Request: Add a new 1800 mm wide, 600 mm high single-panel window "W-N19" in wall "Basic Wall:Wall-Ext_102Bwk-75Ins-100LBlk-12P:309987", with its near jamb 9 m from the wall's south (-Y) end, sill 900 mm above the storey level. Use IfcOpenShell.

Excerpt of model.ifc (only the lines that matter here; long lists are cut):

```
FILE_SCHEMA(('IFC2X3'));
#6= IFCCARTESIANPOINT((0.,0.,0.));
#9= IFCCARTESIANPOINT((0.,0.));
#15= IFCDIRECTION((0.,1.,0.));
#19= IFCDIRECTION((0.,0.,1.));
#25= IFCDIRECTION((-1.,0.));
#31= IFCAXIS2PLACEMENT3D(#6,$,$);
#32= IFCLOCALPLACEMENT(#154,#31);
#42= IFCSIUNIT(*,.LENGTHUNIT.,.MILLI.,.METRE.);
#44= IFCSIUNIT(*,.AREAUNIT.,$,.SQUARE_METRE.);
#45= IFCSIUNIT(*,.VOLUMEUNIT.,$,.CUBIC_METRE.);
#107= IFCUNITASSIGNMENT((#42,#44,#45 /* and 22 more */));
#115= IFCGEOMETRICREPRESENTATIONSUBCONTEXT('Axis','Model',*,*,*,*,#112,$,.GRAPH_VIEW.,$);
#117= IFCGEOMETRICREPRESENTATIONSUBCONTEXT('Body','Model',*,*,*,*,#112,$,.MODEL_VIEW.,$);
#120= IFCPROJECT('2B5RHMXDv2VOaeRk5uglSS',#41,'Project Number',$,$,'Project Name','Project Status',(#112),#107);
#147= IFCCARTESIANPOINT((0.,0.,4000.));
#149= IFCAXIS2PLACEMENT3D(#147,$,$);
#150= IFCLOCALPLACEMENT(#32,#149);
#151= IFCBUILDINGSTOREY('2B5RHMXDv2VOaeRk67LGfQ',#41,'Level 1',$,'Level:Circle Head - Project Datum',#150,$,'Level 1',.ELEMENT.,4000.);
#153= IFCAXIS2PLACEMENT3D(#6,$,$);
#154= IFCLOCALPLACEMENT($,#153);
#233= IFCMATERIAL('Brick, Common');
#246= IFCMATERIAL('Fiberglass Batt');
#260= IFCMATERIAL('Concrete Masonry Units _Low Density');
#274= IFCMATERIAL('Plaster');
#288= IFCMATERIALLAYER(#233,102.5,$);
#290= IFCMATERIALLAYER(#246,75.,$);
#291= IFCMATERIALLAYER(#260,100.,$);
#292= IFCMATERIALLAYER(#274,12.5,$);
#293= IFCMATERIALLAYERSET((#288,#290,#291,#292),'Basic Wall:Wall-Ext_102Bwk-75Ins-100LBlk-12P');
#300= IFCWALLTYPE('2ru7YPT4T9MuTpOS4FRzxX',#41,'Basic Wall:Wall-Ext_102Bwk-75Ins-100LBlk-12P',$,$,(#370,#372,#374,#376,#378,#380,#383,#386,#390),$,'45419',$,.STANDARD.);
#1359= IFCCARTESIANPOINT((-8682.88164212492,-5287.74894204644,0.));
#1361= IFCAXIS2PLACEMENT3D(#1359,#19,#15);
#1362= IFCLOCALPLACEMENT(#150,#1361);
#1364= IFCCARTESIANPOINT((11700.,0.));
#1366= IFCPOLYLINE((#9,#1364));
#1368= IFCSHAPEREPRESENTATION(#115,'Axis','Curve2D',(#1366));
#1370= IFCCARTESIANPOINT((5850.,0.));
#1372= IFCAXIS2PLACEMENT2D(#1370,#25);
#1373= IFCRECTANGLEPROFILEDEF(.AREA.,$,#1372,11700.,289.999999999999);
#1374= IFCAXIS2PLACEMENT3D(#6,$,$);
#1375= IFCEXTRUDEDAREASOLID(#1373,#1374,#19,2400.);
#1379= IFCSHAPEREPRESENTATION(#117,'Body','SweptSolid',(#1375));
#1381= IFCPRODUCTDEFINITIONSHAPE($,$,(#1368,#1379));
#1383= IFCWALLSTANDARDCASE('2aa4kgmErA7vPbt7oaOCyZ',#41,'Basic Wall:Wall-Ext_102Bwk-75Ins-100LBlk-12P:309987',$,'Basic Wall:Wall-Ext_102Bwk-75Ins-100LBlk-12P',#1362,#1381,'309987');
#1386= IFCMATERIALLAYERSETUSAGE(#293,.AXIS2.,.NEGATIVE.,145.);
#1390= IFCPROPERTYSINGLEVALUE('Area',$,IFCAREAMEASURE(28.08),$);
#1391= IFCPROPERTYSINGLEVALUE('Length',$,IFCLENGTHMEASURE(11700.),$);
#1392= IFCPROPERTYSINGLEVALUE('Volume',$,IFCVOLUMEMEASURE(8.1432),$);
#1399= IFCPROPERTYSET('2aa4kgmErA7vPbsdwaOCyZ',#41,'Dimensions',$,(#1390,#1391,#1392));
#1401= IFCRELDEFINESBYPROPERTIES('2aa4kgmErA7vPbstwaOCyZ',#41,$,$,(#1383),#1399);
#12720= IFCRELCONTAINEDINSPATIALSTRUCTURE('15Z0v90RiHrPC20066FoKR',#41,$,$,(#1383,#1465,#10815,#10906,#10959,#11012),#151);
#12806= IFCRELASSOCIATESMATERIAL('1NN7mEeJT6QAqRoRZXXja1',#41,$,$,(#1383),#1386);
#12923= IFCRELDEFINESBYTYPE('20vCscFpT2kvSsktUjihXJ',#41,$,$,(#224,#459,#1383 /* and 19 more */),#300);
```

```python
import numpy as np
import ifcopenshell
import ifcopenshell.api.feature
import ifcopenshell.api.geometry
import ifcopenshell.api.pset
import ifcopenshell.api.root
import ifcopenshell.api.spatial
import ifcopenshell.api.type
import ifcopenshell.geom
import ifcopenshell.util.element
import ifcopenshell.util.placement
import ifcopenshell.util.representation
import ifcopenshell.util.shape
import ifcopenshell.util.unit

model = ifcopenshell.open("model.ifc")
unit_scale = ifcopenshell.util.unit.calculate_unit_scale(model)
area_scale = ifcopenshell.util.unit.calculate_unit_scale(model, "AREAUNIT")
volume_scale = ifcopenshell.util.unit.calculate_unit_scale(model, "VOLUMEUNIT")
settings = ifcopenshell.geom.settings()


def volume(element):
    """Net volume in cubic metres, openings subtracted."""
    shape = ifcopenshell.geom.create_shape(settings, element)
    return ifcopenshell.util.shape.get_volume(shape.geometry)


wall = model.by_guid("2aa4kgmErA7vPbt7oaOCyZ")
storey = ifcopenshell.util.element.get_container(wall, ifc_class="IfcBuildingStorey")
context = ifcopenshell.util.representation.get_context(model, "Model", "Body", "MODEL_VIEW")
before = volume(wall)

width, height, from_end, sill = 1.8, 0.6, 9, 0.9  # metres

# The wall runs along its own X axis, and the end named is its -X end.
wall_shape = ifcopenshell.geom.create_shape(settings, wall)
x, y, z = ifcopenshell.util.shape.get_vertices(wall_shape.geometry).T
start = x.min() + from_end
face, thickness = float(y.min()), float(y.max() - y.min())
wall_matrix = ifcopenshell.util.placement.get_local_placement(wall.ObjectPlacement)
level = ifcopenshell.util.placement.get_local_placement(storey.ObjectPlacement)[2, 3]


def in_wall(x, y):
    """Placement at x, y metres in the wall's axes, at sill height."""
    matrix = wall_matrix.copy()
    matrix[:, 3] = wall_matrix @ np.array([x / unit_scale, y / unit_scale, 0.0, 1.0])
    matrix[2, 3] = level + sill / unit_scale
    return matrix


# Opening: a box that overshoots both wall faces by 50 mm.
opening = ifcopenshell.api.root.create_entity(model, ifc_class="IfcOpeningElement")
box = ifcopenshell.api.geometry.add_wall_representation(
    model, context=context, length=width, height=height, thickness=thickness + 0.1
)
ifcopenshell.api.geometry.assign_representation(model, product=opening, representation=box)
ifcopenshell.api.geometry.edit_object_placement(model, product=opening, matrix=in_wall(start, face - 0.05), is_si=False)
ifcopenshell.api.feature.add_feature(model, feature=opening, element=wall)

window = ifcopenshell.api.root.create_entity(model, ifc_class="IfcWindow", name="W-N19")
window.OverallWidth, window.OverallHeight = width / unit_scale, height / unit_scale
body = ifcopenshell.api.geometry.add_window_representation(
    model,
    context=context,
    overall_width=window.OverallWidth,
    overall_height=window.OverallHeight,
    partition_type="SINGLE_PANEL",
)
ifcopenshell.api.geometry.assign_representation(model, product=window, representation=body)
ifcopenshell.api.spatial.assign_container(model, products=[window], relating_structure=storey)
fills = ifcopenshell.api.feature.add_filling(model, opening=opening, element=window)
fills.OwnerHistory = window.OwnerHistory  # required in IFC2X3

# IFC2X3 keeps the operation on the window style.
style = ifcopenshell.api.root.create_entity(model, ifc_class="IfcWindowStyle", name="W-N19")
style.OperationType, style.ConstructionType = "SINGLE_PANEL", "NOTDEFINED"
style.ParameterTakesPrecedence = style.Sizeable = False
ifcopenshell.api.type.assign_type(model, related_objects=[window], relating_type=style)

# Centre the window in the wall's thickness.
ifcopenshell.api.geometry.edit_object_placement(model, product=window, matrix=in_wall(start, face), is_si=False)
window_shape = ifcopenshell.geom.create_shape(settings, window)
depth = ifcopenshell.util.shape.get_vertices(window_shape.geometry)[:, 1]
offset = face + thickness / 2 - (depth.min() + depth.max()) / 2
ifcopenshell.api.geometry.edit_object_placement(model, product=window, matrix=in_wall(start, offset), is_si=False)

after = volume(wall)

# Update the wall's stored quantities.
pset = model.by_id(ifcopenshell.util.element.get_pset(wall, "Dimensions", should_inherit=False)["id"])
ifcopenshell.api.pset.edit_pset(model, pset=pset, properties={
    "Area": model.create_entity("IfcAreaMeasure", after / thickness / area_scale),
    "Volume": model.create_entity("IfcVolumeMeasure", after / volume_scale),
})

print(f"wall volume {before:.3f} -> {after:.3f} m3")

model.write("model_edited.ifc")
```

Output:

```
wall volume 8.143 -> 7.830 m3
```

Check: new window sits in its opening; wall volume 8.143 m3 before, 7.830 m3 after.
